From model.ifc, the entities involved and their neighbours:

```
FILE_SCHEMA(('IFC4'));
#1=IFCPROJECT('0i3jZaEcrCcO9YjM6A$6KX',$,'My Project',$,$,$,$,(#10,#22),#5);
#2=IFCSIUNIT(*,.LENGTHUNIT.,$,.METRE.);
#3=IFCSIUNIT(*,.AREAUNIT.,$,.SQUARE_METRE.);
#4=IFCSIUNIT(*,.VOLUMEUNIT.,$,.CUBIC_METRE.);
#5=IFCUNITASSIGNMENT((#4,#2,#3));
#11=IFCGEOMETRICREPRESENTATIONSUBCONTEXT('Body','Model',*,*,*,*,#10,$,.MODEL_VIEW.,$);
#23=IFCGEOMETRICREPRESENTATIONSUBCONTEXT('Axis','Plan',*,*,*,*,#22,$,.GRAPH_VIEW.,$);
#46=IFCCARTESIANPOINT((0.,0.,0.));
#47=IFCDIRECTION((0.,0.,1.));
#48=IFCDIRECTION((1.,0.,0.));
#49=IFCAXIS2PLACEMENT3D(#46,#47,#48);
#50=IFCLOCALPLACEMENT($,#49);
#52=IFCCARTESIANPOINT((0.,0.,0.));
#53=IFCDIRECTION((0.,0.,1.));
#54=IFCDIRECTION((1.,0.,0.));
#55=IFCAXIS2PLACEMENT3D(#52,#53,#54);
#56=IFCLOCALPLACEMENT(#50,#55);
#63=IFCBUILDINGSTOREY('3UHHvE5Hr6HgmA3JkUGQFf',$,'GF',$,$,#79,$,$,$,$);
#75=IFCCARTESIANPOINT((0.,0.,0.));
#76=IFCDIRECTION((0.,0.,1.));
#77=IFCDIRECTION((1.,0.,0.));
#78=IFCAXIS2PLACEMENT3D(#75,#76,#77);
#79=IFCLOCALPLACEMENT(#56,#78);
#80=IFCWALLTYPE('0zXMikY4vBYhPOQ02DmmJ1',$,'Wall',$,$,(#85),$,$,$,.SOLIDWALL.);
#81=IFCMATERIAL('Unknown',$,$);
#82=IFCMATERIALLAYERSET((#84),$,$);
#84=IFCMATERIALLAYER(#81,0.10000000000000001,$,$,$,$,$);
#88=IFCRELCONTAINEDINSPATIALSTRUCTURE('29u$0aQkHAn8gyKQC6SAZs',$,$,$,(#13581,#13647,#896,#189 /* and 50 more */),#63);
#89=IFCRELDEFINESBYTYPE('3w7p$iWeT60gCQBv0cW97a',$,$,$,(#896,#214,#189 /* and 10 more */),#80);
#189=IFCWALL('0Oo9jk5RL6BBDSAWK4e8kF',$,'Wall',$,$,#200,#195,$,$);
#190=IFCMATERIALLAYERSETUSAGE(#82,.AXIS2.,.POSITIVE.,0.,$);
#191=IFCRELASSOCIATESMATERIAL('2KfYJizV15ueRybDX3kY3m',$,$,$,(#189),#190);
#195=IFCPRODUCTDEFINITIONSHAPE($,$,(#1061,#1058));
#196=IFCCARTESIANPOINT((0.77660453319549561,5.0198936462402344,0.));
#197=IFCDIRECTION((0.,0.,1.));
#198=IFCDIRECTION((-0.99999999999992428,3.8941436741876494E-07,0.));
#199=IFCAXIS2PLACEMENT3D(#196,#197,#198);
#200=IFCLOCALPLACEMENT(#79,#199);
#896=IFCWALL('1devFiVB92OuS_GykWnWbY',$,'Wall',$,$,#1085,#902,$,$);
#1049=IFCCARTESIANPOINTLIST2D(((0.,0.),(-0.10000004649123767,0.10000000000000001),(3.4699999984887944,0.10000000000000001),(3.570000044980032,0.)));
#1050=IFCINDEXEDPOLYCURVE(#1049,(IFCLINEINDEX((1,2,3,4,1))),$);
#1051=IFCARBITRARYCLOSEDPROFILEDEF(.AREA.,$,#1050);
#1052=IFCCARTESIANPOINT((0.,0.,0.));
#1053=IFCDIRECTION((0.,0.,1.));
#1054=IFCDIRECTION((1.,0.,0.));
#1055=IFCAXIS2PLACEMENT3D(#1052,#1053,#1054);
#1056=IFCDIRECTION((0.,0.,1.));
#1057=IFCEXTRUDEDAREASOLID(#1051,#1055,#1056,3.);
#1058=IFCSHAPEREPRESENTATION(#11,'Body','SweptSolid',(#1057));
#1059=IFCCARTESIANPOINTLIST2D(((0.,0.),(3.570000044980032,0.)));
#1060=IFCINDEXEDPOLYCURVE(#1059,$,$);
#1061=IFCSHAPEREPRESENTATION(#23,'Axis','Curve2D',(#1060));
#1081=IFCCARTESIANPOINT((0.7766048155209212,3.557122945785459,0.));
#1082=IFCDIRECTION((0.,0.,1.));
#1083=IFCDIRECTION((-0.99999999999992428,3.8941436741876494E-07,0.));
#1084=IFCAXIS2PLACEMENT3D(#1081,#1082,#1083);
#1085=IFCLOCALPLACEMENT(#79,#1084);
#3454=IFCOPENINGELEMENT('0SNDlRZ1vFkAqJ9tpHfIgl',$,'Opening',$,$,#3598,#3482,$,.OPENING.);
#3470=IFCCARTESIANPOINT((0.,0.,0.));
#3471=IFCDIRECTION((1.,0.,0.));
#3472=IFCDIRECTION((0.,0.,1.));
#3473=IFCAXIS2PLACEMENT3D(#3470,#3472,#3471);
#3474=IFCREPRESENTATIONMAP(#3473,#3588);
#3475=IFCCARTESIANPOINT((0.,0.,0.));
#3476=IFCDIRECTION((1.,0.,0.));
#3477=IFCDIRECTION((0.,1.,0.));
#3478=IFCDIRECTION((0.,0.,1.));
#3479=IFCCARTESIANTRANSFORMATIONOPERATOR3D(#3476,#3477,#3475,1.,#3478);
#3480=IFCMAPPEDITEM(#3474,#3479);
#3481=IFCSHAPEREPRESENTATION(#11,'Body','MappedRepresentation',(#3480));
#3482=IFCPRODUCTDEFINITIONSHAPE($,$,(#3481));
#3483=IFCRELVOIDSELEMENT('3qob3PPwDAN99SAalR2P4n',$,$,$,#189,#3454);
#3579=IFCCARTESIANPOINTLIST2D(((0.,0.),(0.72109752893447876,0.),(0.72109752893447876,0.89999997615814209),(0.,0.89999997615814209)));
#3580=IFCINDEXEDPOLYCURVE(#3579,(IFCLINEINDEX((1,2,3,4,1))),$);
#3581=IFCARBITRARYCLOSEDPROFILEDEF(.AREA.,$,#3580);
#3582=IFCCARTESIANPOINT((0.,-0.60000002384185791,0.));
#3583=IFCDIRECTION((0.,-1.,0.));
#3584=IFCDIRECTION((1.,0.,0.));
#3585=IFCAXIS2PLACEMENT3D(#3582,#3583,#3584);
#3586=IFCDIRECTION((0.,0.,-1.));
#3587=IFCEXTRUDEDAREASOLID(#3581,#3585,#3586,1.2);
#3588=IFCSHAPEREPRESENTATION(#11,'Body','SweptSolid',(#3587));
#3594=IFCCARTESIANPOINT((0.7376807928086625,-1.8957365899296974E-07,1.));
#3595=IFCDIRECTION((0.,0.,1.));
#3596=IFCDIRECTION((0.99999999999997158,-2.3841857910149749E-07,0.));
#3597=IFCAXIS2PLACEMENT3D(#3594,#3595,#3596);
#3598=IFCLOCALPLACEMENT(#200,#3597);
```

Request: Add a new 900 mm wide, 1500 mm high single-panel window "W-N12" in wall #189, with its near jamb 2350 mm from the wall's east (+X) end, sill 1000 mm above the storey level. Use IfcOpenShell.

```python
import numpy as np
import ifcopenshell
import ifcopenshell.api.feature
import ifcopenshell.api.geometry
import ifcopenshell.api.root
import ifcopenshell.api.spatial
import ifcopenshell.geom
import ifcopenshell.util.element
import ifcopenshell.util.placement
import ifcopenshell.util.representation
import ifcopenshell.util.shape
import ifcopenshell.util.unit

model = ifcopenshell.open("model.ifc")
unit_scale = ifcopenshell.util.unit.calculate_unit_scale(model)
settings = ifcopenshell.geom.settings()


def volume(element):
    """Net volume in cubic metres, openings subtracted."""
    shape = ifcopenshell.geom.create_shape(settings, element)
    return ifcopenshell.util.shape.get_volume(shape.geometry)


wall = model.by_id(189)
storey = ifcopenshell.util.element.get_container(wall, ifc_class="IfcBuildingStorey")
context = ifcopenshell.util.representation.get_context(model, "Model", "Body", "MODEL_VIEW")
before = volume(wall)

width, height, from_end, sill = 0.9, 1.5, 2.35, 1  # metres

# The wall runs along its own X axis, and the end named is its -X end.
wall_shape = ifcopenshell.geom.create_shape(settings, wall)
x, y, z = ifcopenshell.util.shape.get_vertices(wall_shape.geometry).T
start = x.min() + from_end
face, thickness = float(y.min()), float(y.max() - y.min())
wall_matrix = ifcopenshell.util.placement.get_local_placement(wall.ObjectPlacement)
level = ifcopenshell.util.placement.get_local_placement(storey.ObjectPlacement)[2, 3]


def in_wall(x, y):
    """Placement at x, y metres in the wall's axes, at sill height."""
    matrix = wall_matrix.copy()
    matrix[:, 3] = wall_matrix @ np.array([x / unit_scale, y / unit_scale, 0.0, 1.0])
    matrix[2, 3] = level + sill / unit_scale
    return matrix


# Opening: a box that overshoots both wall faces by 50 mm.
opening = ifcopenshell.api.root.create_entity(model, ifc_class="IfcOpeningElement", predefined_type="OPENING")
box = ifcopenshell.api.geometry.add_wall_representation(
    model, context=context, length=width, height=height, thickness=thickness + 0.1
)
ifcopenshell.api.geometry.assign_representation(model, product=opening, representation=box)
ifcopenshell.api.geometry.edit_object_placement(model, product=opening, matrix=in_wall(start, face - 0.05), is_si=False)
ifcopenshell.api.feature.add_feature(model, feature=opening, element=wall)

window = ifcopenshell.api.root.create_entity(model, ifc_class="IfcWindow", name="W-N12", predefined_type="WINDOW")
window.OverallWidth, window.OverallHeight = width / unit_scale, height / unit_scale
window.PartitioningType = "SINGLE_PANEL"
body = ifcopenshell.api.geometry.add_window_representation(
    model,
    context=context,
    overall_width=window.OverallWidth,
    overall_height=window.OverallHeight,
    partition_type="SINGLE_PANEL",
)
ifcopenshell.api.geometry.assign_representation(model, product=window, representation=body)
ifcopenshell.api.spatial.assign_container(model, products=[window], relating_structure=storey)
ifcopenshell.api.feature.add_filling(model, opening=opening, element=window)

# Centre the window in the wall's thickness.
ifcopenshell.api.geometry.edit_object_placement(model, product=window, matrix=in_wall(start, face), is_si=False)
window_shape = ifcopenshell.geom.create_shape(settings, window)
depth = ifcopenshell.util.shape.get_vertices(window_shape.geometry)[:, 1]
offset = face + thickness / 2 - (depth.min() + depth.max()) / 2
ifcopenshell.api.geometry.edit_object_placement(model, product=window, matrix=in_wall(start, offset), is_si=False)

after = volume(wall)

print(f"wall volume {before:.3f} -> {after:.3f} m3")

model.write("model_edited.ifc")
```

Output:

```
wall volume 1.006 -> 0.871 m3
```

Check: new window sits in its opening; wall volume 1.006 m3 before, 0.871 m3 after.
